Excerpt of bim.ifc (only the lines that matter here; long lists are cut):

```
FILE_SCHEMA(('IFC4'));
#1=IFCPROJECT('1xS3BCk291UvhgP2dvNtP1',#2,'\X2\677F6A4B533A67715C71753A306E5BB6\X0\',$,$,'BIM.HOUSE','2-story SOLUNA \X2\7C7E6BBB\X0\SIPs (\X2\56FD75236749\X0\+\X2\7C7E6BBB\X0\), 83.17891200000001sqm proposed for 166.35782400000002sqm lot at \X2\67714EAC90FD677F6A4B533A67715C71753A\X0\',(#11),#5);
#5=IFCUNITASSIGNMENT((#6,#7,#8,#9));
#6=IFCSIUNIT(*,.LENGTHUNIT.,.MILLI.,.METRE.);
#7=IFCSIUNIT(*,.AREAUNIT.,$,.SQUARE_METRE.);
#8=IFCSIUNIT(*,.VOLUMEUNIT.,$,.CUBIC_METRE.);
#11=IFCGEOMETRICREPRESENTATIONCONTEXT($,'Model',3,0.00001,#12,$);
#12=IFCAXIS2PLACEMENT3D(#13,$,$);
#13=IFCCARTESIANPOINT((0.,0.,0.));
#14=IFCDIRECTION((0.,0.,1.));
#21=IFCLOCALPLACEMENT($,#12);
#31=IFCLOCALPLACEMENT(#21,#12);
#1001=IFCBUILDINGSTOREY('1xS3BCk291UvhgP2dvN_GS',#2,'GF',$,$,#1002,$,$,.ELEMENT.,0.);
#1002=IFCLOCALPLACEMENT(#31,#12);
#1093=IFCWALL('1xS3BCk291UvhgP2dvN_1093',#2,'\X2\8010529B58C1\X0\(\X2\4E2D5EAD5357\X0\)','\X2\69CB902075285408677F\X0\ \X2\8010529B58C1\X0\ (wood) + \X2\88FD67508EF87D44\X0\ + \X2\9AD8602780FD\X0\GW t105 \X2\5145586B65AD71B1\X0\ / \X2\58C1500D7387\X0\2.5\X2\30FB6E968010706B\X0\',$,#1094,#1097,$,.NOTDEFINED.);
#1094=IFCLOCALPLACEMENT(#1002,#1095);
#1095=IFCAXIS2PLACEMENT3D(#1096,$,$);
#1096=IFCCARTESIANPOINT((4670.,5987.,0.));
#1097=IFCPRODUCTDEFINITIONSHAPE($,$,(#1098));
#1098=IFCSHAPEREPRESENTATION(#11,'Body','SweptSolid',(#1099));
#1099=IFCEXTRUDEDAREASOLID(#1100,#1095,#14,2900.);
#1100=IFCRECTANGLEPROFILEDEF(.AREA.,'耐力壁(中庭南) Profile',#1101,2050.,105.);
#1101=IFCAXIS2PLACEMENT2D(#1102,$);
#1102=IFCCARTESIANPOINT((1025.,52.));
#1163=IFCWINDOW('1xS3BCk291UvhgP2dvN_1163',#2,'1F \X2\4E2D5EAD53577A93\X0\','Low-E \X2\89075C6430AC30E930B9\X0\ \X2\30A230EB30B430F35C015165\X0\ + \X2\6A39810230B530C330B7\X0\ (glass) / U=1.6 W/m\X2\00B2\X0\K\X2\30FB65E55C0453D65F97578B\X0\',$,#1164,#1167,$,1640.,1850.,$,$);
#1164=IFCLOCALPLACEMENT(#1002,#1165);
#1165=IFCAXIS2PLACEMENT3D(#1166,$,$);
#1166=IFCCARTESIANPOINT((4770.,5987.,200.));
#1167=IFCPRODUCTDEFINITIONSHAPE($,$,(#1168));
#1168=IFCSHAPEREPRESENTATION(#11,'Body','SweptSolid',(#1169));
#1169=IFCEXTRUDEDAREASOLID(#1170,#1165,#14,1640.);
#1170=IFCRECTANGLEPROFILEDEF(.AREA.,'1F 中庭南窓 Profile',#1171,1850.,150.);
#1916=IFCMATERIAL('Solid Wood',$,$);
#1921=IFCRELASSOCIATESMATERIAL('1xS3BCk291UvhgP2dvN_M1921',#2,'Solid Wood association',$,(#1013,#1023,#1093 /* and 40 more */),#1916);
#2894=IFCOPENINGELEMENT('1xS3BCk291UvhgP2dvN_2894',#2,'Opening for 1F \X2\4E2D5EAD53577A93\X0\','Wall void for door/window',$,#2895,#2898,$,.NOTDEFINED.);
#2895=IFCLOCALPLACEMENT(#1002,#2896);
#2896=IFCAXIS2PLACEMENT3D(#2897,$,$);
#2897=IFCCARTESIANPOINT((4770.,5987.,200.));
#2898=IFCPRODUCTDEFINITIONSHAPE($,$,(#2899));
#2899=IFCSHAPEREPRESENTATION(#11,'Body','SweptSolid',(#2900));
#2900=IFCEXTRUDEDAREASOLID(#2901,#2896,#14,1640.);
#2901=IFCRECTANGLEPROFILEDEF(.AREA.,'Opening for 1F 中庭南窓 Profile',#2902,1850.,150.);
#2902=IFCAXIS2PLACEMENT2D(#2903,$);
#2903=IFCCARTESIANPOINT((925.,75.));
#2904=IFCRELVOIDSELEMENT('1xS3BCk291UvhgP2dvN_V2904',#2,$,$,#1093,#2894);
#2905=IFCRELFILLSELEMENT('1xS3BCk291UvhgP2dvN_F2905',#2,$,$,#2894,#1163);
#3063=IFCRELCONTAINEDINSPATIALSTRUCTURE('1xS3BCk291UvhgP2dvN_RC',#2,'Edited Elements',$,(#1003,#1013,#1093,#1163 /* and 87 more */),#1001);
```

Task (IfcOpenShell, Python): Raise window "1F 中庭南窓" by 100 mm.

```python
import numpy as np
import ifcopenshell
import ifcopenshell.api.geometry
import ifcopenshell.util.placement
import ifcopenshell.util.unit

model = ifcopenshell.open("bim.ifc")
unit_scale = ifcopenshell.util.unit.calculate_unit_scale(model)

window = model.by_id(1163)
opening = window.FillsVoids[0].RelatingOpeningElement
dz = 0.1 / unit_scale

shift = np.array([0.0, 0.0, dz])
# The window is not placed relative to its opening, so move both.
for product in (opening, window):
    matrix = ifcopenshell.util.placement.get_local_placement(product.ObjectPlacement)
    matrix[:3, 3] += shift
    ifcopenshell.api.geometry.edit_object_placement(model, product=product, matrix=matrix, is_si=False)

print(f"moved by {dz * unit_scale:+.3f} m")

model.write("bim-out.ifc")
```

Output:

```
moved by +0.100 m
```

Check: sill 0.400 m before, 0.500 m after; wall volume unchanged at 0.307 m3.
